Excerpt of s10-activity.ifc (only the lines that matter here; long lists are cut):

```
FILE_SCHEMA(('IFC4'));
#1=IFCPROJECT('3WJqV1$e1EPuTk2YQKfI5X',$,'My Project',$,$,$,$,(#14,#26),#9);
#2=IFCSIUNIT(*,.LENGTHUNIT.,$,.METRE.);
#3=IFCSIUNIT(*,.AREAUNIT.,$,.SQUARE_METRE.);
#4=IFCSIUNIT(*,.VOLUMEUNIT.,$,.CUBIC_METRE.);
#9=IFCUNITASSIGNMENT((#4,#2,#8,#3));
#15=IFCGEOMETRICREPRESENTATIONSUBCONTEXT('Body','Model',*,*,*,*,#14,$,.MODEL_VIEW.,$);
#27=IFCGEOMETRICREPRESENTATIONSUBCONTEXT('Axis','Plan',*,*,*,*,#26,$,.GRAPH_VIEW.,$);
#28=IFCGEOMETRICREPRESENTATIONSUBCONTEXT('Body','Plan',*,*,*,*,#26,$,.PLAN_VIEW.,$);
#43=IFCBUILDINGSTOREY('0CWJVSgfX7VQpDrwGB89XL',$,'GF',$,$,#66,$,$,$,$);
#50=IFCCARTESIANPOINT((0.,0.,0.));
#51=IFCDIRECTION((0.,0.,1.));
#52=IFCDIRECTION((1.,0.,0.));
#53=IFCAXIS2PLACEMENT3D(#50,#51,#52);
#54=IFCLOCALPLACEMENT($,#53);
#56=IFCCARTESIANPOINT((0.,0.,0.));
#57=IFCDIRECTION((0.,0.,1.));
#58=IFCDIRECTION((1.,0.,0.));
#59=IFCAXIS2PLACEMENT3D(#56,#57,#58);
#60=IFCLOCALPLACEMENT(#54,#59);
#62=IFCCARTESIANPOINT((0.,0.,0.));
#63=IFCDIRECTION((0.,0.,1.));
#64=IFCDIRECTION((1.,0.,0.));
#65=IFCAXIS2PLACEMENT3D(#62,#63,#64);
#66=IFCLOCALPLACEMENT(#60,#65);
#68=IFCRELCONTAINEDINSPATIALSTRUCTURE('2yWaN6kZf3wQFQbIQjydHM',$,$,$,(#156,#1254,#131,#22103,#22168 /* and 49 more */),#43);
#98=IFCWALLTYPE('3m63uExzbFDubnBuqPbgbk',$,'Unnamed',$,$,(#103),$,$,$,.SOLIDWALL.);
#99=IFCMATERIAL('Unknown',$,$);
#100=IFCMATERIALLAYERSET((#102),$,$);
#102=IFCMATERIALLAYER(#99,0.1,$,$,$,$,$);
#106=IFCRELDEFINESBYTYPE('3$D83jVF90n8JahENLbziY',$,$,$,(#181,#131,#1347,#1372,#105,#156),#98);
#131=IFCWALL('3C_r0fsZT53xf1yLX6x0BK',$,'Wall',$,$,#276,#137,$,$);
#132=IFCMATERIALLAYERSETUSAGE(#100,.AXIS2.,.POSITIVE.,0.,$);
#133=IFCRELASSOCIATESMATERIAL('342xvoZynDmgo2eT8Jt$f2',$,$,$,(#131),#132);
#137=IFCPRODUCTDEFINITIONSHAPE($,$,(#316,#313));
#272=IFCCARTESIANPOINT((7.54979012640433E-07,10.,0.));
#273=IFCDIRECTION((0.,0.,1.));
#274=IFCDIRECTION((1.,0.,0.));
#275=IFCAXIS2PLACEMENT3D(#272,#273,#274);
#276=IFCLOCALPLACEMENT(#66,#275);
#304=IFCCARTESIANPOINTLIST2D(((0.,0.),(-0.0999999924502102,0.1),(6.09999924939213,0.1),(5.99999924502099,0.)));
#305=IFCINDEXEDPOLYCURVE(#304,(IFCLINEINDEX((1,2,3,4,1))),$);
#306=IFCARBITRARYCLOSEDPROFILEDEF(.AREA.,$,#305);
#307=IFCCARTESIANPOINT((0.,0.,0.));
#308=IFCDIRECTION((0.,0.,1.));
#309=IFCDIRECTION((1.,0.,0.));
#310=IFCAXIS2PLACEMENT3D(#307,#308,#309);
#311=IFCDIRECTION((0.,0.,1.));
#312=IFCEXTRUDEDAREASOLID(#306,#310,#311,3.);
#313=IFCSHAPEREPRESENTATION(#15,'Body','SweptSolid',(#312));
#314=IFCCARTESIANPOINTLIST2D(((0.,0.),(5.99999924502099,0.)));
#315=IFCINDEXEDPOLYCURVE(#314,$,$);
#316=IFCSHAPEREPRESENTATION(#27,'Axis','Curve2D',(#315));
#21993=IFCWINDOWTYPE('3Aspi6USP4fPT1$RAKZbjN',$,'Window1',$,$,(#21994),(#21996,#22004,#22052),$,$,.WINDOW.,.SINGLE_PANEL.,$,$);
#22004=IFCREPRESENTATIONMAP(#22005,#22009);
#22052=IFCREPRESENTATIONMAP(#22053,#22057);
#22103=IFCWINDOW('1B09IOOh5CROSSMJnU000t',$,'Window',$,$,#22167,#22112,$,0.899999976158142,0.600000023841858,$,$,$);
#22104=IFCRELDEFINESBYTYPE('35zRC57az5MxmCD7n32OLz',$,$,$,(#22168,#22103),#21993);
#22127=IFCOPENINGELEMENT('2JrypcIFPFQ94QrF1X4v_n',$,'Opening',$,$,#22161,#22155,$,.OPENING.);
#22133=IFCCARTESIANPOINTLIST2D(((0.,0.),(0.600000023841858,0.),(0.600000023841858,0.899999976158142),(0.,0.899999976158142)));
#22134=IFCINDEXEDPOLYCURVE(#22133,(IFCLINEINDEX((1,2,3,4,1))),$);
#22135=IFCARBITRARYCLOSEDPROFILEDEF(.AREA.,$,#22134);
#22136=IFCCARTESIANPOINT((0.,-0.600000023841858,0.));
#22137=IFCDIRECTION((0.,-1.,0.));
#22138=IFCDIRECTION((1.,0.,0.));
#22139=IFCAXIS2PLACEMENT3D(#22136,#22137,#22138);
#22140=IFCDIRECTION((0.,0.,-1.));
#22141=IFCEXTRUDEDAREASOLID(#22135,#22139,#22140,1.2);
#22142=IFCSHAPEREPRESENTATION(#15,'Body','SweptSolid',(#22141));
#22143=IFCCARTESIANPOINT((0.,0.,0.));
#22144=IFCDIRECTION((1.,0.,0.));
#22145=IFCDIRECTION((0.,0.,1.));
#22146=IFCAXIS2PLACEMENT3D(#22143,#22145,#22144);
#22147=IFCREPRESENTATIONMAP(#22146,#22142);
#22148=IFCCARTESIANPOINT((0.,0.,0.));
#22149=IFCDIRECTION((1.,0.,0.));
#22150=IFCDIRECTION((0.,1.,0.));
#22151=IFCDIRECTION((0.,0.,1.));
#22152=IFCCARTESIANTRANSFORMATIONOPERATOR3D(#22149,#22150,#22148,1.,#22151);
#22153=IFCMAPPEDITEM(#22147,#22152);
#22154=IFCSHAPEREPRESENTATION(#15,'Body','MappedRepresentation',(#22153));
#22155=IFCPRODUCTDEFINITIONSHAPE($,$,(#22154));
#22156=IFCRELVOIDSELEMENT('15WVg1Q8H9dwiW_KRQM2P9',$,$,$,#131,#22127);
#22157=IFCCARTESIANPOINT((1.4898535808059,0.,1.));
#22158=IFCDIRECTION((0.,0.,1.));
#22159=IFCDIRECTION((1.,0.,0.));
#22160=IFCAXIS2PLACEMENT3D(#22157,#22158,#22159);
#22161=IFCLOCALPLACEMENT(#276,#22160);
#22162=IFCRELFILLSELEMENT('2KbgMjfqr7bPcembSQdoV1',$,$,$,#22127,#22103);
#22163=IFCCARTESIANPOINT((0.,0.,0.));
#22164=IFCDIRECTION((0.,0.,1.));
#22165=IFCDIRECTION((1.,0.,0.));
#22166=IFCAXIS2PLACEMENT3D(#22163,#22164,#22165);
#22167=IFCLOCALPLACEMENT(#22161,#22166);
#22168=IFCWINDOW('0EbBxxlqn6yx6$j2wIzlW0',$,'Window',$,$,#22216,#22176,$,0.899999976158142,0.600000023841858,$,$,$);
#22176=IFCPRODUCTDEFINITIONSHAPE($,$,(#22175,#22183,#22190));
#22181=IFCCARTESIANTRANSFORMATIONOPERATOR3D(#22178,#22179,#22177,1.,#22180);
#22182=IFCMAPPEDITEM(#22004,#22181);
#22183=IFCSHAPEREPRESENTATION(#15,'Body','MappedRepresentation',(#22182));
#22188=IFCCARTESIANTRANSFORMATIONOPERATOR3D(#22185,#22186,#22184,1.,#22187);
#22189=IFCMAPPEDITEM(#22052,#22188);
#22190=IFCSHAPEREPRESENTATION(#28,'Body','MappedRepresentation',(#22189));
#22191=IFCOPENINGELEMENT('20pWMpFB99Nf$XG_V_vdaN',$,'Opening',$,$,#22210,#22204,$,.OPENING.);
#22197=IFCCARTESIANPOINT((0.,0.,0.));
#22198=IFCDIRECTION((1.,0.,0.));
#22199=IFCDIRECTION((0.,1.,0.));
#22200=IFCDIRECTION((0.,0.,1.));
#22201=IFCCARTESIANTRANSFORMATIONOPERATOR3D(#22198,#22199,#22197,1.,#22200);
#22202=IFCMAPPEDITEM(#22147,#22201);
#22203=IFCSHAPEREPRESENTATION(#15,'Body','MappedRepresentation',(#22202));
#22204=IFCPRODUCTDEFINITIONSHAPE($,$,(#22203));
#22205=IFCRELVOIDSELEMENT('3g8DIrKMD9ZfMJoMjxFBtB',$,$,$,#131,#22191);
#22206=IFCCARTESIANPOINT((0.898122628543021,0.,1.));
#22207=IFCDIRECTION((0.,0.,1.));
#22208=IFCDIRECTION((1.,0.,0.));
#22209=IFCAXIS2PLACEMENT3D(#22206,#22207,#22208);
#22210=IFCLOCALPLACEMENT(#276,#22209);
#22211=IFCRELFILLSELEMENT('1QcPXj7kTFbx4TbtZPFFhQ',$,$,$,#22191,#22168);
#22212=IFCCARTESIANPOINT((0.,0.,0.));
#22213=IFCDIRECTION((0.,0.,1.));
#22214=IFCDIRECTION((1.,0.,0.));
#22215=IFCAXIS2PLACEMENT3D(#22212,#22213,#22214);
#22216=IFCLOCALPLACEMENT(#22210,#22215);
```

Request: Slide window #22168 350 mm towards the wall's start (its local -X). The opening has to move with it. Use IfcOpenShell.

```python
import ifcopenshell
import ifcopenshell.api.geometry
import ifcopenshell.util.placement
import ifcopenshell.util.unit

model = ifcopenshell.open("s10-activity.ifc")
unit_scale = ifcopenshell.util.unit.calculate_unit_scale(model)

window = model.by_id(22168)
opening = window.FillsVoids[0].RelatingOpeningElement
wall = opening.VoidsElements[0].RelatingBuildingElement

wall_matrix = ifcopenshell.util.placement.get_local_placement(wall.ObjectPlacement)
shift = wall_matrix[:3, 0] * -0.35 / unit_scale
before = ifcopenshell.util.placement.get_local_placement(window.ObjectPlacement)[:3, 3].copy()

# The window is placed relative to its opening, so it follows when the opening moves.
matrix = ifcopenshell.util.placement.get_local_placement(opening.ObjectPlacement)
matrix[:3, 3] += shift
ifcopenshell.api.geometry.edit_object_placement(
    model, product=opening, matrix=matrix, is_si=False, should_transform_children=True
)

after = ifcopenshell.util.placement.get_local_placement(window.ObjectPlacement)[:3, 3]
print("window moved by", (after - before).round(3) + 0.0)

model.write("s10-activity_edited.ifc")
```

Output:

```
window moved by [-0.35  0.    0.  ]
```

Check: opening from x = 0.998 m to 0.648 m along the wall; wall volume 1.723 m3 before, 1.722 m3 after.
